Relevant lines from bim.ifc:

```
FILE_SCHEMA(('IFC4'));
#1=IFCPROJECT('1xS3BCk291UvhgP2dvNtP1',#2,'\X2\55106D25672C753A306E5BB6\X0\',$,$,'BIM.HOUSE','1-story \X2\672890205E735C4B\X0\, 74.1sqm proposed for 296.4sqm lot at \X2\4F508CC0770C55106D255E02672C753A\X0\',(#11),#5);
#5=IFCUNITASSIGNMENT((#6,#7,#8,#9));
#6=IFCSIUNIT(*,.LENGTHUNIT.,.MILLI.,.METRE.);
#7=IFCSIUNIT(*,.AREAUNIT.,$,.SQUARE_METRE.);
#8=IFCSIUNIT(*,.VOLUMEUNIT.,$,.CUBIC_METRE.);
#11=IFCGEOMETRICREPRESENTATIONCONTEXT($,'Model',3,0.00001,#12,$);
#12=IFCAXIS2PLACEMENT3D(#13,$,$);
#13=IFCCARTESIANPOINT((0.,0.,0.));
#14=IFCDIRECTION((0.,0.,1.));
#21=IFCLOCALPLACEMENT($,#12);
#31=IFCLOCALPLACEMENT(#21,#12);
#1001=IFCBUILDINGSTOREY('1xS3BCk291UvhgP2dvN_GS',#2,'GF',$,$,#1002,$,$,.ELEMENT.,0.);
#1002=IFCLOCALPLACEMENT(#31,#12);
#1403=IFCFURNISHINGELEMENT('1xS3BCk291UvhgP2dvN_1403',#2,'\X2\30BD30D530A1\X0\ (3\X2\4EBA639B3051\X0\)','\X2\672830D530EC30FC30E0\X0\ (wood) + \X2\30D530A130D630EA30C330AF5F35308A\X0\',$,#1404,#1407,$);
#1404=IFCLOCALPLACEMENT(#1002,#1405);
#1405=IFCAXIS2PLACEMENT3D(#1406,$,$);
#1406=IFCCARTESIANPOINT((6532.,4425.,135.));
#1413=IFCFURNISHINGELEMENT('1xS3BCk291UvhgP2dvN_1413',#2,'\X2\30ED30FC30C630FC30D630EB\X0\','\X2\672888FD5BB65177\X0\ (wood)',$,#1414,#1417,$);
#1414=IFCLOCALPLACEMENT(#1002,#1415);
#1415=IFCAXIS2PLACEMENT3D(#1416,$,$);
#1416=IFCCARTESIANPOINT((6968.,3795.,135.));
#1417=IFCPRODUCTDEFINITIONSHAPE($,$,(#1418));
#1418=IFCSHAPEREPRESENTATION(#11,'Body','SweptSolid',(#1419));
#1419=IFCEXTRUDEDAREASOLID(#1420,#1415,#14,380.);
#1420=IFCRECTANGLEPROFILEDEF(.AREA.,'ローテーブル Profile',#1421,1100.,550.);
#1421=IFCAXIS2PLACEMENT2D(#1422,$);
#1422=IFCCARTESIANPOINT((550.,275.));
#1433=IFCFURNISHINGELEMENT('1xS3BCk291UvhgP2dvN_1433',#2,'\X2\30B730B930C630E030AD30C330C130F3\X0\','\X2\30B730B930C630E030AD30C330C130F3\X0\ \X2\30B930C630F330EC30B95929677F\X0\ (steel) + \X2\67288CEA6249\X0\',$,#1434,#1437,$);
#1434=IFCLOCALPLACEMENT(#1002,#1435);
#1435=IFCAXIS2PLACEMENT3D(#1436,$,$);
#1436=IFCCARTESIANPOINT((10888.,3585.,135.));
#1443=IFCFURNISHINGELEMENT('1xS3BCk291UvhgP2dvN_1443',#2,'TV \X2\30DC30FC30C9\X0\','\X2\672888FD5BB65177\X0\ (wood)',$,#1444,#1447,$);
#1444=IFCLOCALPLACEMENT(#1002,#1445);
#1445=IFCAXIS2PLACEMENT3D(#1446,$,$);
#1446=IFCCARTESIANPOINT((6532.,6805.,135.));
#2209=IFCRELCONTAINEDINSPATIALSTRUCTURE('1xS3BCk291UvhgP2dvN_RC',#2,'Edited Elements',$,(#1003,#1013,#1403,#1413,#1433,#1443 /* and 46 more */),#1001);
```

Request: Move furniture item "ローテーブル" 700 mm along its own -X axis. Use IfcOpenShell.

```python
import ifcopenshell
import ifcopenshell.api.geometry
import ifcopenshell.util.placement

model = ifcopenshell.open("bim.ifc")

item = model.by_guid("1xS3BCk291UvhgP2dvN_1413")
matrix = ifcopenshell.util.placement.get_local_placement(item.ObjectPlacement)
matrix[:3, 3] -= matrix[:3, 0] * 700.0
ifcopenshell.api.geometry.edit_object_placement(model, product=item, matrix=matrix, is_si=False)

print(ifcopenshell.util.placement.get_local_placement(item.ObjectPlacement).round(3) + 0.0)

model.write("bim_edited.ifc")
```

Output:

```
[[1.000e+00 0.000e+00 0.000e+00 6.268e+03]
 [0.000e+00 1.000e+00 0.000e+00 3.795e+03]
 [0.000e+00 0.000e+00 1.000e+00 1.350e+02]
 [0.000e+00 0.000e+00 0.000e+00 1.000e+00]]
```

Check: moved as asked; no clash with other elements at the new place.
